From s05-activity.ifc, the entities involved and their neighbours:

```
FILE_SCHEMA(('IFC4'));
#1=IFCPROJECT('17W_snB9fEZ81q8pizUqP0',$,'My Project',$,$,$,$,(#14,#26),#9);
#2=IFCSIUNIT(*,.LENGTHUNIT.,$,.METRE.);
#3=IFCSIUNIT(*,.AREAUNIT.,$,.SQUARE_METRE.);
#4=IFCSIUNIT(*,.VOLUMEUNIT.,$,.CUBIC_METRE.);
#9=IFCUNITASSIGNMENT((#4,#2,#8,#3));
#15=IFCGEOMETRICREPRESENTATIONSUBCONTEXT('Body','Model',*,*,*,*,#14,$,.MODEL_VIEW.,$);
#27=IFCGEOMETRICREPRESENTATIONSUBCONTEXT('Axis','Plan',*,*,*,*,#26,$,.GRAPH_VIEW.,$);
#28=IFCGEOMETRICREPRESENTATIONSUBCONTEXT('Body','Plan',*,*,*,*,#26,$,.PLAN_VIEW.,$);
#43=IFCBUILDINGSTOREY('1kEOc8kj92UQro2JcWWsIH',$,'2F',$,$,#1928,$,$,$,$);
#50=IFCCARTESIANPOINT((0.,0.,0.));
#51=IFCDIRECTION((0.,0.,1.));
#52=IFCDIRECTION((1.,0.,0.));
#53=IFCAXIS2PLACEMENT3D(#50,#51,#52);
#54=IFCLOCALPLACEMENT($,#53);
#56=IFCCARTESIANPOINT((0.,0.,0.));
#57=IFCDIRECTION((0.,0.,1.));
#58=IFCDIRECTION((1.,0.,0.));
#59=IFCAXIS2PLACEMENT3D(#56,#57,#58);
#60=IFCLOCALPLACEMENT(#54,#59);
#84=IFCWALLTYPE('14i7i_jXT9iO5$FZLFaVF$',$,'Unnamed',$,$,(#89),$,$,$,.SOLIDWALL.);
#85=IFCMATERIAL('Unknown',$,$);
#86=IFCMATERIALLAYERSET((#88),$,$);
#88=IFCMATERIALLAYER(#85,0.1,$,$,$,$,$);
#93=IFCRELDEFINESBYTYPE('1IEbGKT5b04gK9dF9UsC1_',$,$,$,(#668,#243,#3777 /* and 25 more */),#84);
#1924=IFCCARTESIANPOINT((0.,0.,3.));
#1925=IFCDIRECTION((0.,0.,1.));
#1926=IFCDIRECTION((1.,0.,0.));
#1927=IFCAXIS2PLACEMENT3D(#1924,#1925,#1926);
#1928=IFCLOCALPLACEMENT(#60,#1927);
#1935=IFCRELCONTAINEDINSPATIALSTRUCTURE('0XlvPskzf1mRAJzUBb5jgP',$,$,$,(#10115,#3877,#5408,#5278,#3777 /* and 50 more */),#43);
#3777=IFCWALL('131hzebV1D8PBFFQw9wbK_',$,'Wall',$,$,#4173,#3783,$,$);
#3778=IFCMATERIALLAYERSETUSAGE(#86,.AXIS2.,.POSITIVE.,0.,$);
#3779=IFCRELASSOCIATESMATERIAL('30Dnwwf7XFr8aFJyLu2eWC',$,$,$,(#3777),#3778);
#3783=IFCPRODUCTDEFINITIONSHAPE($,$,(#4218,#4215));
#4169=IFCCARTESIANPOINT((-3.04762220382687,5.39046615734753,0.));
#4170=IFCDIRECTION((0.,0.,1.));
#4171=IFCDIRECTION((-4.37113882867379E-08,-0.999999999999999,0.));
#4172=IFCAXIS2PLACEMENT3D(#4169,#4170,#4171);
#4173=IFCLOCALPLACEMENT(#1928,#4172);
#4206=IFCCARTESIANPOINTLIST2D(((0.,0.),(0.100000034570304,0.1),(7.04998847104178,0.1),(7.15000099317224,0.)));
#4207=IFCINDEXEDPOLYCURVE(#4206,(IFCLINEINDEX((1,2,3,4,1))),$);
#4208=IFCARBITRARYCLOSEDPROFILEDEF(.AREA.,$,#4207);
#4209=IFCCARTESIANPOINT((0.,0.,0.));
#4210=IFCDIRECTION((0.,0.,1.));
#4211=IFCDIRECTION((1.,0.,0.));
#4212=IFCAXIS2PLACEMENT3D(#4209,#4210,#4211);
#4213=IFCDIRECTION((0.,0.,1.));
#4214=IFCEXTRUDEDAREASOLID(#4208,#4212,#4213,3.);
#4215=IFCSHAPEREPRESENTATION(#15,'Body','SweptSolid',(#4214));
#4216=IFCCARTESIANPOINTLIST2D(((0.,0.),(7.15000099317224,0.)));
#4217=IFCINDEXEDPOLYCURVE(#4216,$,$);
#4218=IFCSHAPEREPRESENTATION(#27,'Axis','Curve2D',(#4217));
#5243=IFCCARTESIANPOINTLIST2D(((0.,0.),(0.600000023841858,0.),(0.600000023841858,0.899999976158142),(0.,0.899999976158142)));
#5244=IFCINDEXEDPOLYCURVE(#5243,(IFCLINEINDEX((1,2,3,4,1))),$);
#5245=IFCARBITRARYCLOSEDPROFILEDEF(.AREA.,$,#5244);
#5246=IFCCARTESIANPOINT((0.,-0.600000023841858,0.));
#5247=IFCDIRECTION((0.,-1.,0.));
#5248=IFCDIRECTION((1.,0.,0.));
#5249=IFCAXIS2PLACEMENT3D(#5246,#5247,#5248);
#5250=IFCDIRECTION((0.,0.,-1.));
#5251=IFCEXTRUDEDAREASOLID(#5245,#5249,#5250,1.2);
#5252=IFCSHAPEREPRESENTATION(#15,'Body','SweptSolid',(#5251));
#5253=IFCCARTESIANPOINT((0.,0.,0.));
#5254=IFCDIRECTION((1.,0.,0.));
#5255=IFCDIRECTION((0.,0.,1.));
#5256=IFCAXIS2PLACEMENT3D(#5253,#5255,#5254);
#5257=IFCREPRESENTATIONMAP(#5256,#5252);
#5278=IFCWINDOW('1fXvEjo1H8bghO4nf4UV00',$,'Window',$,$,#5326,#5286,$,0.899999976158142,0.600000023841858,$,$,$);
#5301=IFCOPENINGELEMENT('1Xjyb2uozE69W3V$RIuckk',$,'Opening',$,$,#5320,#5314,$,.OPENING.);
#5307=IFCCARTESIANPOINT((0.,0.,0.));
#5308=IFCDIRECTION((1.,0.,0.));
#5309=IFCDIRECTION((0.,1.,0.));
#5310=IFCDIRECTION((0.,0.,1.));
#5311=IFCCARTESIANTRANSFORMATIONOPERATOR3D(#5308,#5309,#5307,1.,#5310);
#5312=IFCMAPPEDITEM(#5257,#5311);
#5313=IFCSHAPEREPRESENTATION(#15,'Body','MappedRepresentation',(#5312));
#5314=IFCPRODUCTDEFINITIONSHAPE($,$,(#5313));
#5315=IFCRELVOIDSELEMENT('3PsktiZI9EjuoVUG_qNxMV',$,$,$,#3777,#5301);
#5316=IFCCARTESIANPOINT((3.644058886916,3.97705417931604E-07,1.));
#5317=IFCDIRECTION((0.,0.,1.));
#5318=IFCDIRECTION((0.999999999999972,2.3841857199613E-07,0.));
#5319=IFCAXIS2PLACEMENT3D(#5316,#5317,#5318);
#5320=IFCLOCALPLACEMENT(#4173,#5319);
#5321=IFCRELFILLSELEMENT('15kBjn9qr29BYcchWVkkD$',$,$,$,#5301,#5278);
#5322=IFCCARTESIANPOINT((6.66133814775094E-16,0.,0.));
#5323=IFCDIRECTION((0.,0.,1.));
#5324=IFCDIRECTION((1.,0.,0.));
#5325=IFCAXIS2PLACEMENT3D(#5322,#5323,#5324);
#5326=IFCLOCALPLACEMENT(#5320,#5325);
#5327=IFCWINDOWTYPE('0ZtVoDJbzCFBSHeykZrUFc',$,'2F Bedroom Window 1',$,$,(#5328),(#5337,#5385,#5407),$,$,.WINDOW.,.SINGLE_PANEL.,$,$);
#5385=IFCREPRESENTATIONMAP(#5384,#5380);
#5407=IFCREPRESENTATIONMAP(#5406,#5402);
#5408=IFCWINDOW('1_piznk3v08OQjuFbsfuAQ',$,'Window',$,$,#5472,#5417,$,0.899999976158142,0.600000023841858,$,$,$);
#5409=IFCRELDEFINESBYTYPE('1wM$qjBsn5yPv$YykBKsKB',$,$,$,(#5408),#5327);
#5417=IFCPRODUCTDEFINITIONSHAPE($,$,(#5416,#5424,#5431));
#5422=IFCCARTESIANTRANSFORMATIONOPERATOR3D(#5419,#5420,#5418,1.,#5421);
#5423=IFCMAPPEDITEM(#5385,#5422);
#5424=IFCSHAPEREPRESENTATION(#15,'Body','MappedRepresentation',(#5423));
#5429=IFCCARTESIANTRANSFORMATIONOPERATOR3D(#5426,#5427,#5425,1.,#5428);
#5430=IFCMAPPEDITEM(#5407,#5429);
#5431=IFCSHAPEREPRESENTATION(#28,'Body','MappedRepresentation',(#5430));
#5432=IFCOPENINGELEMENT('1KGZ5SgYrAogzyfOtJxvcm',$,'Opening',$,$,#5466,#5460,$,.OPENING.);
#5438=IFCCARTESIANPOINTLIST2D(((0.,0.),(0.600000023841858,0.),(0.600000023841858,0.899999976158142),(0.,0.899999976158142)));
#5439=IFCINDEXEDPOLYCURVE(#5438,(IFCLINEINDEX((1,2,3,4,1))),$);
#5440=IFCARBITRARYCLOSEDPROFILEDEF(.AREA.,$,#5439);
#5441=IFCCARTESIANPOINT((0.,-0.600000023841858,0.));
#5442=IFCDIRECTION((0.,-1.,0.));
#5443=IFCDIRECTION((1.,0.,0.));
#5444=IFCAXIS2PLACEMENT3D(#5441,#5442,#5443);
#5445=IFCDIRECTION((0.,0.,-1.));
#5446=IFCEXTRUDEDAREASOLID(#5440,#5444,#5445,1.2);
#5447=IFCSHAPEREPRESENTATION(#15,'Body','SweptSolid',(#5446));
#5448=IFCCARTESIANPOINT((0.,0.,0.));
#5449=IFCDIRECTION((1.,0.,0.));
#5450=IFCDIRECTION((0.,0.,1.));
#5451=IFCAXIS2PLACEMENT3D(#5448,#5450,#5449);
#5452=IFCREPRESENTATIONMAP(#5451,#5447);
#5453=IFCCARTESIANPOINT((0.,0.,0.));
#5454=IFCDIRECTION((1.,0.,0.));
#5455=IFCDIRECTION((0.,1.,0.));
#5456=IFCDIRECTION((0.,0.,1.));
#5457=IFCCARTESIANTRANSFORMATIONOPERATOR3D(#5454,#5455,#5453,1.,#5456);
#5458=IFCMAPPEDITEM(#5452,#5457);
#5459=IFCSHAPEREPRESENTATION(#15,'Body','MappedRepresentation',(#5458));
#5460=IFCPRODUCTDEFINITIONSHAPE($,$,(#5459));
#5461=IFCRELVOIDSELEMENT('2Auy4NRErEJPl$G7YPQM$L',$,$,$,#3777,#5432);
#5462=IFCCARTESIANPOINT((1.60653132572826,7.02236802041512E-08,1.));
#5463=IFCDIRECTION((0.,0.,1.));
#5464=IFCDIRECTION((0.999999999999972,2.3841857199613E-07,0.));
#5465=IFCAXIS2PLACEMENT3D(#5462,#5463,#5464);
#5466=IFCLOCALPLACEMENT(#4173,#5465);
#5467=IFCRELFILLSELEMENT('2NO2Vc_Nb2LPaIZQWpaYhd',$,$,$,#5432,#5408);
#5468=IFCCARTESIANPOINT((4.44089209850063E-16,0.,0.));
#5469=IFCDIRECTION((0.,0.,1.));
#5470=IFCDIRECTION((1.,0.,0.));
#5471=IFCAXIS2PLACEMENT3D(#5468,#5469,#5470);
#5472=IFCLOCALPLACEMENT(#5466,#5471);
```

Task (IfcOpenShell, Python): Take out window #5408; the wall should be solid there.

```python
import ifcopenshell
import ifcopenshell.api.feature
import ifcopenshell.api.root
import ifcopenshell.geom
import ifcopenshell.util.shape

model = ifcopenshell.open("s05-activity.ifc")
settings = ifcopenshell.geom.settings()


def volume(element):
    """Net volume in cubic metres, openings subtracted."""
    shape = ifcopenshell.geom.create_shape(settings, element)
    return ifcopenshell.util.shape.get_volume(shape.geometry)


window = model.by_guid("1_piznk3v08OQjuFbsfuAQ")
opening = window.FillsVoids[0].RelatingOpeningElement
wall = opening.VoidsElements[0].RelatingBuildingElement
before = volume(wall)

ifcopenshell.api.root.remove_product(model, product=window)
ifcopenshell.api.feature.remove_feature(model, feature=opening)

after = volume(wall)

print(f"wall volume {before:.3f} -> {after:.3f} m3")

model.write("s05-activity_edited.ifc")
```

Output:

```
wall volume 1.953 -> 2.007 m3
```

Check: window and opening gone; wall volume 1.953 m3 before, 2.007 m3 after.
